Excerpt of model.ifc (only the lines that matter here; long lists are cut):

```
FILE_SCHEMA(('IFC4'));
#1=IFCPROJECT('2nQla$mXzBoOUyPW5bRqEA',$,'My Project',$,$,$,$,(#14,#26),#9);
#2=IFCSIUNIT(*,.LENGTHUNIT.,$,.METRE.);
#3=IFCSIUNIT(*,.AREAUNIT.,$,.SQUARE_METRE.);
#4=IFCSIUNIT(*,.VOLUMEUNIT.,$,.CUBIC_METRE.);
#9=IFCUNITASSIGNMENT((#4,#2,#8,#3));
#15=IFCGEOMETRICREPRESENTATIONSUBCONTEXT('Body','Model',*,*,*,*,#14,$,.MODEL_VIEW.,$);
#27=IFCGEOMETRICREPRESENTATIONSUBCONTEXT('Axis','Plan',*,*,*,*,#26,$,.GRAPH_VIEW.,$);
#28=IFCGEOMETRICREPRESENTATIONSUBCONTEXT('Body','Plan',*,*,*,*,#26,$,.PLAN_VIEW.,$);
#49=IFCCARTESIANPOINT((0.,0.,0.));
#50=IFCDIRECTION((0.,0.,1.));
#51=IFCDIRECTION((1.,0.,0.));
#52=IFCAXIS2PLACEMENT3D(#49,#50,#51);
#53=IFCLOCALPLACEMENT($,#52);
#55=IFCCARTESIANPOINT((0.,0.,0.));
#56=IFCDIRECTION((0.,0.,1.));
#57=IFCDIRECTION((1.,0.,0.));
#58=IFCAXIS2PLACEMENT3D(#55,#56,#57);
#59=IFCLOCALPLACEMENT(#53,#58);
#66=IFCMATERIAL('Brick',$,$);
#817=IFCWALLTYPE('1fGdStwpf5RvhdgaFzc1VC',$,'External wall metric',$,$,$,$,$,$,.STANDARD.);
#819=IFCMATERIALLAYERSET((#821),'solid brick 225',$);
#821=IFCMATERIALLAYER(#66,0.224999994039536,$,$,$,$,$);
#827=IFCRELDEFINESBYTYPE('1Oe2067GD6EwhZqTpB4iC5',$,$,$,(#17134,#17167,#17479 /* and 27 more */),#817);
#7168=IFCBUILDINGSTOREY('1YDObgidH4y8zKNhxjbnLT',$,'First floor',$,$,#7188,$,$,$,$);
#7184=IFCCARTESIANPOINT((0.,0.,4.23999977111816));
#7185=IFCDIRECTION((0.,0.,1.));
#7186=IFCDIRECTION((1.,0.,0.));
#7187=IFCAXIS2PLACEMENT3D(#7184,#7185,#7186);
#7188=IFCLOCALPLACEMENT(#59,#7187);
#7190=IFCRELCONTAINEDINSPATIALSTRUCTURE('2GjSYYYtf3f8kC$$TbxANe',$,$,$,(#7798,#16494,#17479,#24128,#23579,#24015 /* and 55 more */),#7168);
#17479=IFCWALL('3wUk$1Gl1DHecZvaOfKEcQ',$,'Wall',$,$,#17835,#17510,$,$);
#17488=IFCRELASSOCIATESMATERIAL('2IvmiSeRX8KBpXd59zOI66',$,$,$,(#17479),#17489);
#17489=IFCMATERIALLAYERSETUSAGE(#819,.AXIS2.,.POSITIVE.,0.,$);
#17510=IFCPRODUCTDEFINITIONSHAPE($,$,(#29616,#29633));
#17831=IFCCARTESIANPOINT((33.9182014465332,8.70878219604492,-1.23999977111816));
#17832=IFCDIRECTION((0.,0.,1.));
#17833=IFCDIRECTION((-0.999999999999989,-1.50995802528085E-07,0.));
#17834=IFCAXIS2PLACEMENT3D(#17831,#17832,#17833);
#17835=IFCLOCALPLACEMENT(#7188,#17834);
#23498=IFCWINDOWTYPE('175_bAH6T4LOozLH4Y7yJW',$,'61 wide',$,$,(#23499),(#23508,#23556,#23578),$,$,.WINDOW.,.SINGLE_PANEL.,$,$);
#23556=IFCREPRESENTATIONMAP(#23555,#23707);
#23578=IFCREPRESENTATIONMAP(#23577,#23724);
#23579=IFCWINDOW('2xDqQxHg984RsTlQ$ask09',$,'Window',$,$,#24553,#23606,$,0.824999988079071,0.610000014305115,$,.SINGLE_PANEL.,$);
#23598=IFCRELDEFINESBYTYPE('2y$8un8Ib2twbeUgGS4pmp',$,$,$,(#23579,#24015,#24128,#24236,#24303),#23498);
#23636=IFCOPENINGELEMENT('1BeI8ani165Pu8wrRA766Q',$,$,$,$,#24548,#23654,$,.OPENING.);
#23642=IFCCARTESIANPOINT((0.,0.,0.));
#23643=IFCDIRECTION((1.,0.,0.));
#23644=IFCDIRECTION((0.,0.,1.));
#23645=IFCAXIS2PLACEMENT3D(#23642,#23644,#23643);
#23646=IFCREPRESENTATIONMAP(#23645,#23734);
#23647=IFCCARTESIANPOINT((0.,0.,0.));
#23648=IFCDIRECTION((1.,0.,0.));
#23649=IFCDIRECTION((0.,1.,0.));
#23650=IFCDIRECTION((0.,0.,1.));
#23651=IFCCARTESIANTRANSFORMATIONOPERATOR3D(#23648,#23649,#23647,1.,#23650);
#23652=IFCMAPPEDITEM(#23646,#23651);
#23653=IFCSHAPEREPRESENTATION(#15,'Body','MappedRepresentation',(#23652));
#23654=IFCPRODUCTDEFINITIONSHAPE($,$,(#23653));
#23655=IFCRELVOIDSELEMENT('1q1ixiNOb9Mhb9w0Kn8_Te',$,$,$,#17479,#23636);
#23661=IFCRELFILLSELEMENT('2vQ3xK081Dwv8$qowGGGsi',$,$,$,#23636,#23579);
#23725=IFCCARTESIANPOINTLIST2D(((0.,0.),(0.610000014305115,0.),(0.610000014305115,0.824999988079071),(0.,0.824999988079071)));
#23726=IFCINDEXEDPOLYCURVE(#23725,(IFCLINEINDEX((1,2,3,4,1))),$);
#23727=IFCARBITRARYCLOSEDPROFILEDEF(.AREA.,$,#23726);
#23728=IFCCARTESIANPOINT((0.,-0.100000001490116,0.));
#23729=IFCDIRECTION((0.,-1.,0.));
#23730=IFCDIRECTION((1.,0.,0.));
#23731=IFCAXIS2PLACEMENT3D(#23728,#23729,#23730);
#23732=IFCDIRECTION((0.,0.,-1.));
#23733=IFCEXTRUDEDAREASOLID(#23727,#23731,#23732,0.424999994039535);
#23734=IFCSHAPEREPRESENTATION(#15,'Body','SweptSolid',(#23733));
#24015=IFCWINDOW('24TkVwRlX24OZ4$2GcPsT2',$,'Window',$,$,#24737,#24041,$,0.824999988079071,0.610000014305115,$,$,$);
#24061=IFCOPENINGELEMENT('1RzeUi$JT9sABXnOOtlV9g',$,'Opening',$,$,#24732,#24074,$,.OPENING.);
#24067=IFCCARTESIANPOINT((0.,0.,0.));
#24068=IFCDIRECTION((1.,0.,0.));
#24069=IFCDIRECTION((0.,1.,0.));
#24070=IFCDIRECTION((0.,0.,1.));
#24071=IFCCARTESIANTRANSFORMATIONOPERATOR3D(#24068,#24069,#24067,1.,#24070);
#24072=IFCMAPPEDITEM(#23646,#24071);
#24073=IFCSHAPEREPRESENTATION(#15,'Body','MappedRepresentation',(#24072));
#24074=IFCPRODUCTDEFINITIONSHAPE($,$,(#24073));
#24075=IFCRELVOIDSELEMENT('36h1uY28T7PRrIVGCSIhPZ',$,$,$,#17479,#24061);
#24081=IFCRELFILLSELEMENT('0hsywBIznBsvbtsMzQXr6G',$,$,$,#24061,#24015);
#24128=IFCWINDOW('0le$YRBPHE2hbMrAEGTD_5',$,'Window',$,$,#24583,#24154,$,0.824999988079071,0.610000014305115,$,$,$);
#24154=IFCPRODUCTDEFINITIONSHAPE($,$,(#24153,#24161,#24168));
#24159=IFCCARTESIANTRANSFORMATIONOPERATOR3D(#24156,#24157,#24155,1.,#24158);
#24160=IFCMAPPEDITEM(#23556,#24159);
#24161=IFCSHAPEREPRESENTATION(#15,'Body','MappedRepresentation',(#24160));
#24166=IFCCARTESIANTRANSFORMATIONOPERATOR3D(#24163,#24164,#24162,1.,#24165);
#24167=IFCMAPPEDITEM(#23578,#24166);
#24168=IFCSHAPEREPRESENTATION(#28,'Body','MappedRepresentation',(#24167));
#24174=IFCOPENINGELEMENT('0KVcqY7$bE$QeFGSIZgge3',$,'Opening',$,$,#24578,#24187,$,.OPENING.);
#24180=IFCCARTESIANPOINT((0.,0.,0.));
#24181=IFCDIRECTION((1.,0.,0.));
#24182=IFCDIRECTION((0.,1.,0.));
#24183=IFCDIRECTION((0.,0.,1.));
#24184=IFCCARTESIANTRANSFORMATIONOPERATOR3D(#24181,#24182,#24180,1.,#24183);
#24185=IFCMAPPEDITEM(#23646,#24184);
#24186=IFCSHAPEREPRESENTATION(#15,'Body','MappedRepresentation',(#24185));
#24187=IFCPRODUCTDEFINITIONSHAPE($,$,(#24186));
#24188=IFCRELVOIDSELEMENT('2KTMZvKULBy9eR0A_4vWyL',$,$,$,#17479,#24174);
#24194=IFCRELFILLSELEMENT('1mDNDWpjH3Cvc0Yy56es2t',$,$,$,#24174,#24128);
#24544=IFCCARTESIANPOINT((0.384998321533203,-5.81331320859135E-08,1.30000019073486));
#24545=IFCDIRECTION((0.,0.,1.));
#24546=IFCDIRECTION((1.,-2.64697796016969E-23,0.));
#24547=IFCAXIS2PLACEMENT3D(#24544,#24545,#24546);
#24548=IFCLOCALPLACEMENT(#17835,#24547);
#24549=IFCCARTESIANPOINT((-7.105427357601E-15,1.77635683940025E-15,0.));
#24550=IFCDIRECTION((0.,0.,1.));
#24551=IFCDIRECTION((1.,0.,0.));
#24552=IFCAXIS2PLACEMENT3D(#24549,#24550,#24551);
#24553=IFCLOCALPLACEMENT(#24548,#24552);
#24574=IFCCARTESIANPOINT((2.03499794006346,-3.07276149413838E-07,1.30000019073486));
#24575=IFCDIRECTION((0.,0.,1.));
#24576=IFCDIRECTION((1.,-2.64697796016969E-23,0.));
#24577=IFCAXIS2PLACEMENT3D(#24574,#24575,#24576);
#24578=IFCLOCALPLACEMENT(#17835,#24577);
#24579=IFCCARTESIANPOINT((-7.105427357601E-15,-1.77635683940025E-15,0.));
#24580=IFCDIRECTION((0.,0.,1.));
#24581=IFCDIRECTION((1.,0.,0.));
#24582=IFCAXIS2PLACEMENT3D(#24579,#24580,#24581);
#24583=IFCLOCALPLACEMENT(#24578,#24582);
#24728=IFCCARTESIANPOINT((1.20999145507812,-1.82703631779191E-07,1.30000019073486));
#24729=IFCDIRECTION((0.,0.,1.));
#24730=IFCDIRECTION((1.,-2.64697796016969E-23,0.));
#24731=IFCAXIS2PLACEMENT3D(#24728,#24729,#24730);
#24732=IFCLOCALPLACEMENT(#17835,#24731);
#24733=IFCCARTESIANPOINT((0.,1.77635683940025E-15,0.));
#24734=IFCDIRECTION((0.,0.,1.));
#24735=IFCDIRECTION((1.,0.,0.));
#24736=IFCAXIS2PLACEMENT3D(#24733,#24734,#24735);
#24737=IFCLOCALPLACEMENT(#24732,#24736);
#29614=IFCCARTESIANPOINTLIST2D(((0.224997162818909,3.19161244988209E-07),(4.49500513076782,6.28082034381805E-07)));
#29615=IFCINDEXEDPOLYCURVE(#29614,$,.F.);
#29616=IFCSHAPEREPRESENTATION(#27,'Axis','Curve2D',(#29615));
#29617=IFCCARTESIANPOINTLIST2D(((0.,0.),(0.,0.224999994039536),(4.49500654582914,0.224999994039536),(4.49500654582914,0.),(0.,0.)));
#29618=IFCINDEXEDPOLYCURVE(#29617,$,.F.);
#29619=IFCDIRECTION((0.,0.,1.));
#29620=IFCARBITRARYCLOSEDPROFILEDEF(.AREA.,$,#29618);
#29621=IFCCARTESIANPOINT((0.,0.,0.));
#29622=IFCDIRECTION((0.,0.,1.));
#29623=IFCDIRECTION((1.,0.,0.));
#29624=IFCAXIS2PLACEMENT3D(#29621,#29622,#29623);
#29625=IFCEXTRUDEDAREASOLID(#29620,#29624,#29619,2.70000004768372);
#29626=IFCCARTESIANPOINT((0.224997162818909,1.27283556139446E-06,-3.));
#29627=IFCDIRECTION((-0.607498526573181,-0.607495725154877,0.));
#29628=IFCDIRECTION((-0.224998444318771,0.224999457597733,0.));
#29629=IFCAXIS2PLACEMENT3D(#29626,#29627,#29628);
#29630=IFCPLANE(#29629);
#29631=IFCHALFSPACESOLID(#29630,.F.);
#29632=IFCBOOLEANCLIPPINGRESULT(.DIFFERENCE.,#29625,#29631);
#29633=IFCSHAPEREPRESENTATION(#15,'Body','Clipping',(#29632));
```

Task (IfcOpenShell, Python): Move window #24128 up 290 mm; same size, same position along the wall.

```python
import numpy as np
import ifcopenshell
import ifcopenshell.api.geometry
import ifcopenshell.util.placement
import ifcopenshell.util.unit

model = ifcopenshell.open("model.ifc")
unit_scale = ifcopenshell.util.unit.calculate_unit_scale(model)

window = model.by_guid("0le$YRBPHE2hbMrAEGTD_5")
opening = window.FillsVoids[0].RelatingOpeningElement
dz = 0.29

shift = np.array([0.0, 0.0, dz])
# The window is placed relative to its opening, so it follows when the opening moves.
matrix = ifcopenshell.util.placement.get_local_placement(opening.ObjectPlacement)
matrix[:3, 3] += shift
ifcopenshell.api.geometry.edit_object_placement(
    model, product=opening, matrix=matrix, is_si=False, should_transform_children=True
)

print(f"moved by {dz * unit_scale:+.3f} m")

model.write("model_rev.ifc")
```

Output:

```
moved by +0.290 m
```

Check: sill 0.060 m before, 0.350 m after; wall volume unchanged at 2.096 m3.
